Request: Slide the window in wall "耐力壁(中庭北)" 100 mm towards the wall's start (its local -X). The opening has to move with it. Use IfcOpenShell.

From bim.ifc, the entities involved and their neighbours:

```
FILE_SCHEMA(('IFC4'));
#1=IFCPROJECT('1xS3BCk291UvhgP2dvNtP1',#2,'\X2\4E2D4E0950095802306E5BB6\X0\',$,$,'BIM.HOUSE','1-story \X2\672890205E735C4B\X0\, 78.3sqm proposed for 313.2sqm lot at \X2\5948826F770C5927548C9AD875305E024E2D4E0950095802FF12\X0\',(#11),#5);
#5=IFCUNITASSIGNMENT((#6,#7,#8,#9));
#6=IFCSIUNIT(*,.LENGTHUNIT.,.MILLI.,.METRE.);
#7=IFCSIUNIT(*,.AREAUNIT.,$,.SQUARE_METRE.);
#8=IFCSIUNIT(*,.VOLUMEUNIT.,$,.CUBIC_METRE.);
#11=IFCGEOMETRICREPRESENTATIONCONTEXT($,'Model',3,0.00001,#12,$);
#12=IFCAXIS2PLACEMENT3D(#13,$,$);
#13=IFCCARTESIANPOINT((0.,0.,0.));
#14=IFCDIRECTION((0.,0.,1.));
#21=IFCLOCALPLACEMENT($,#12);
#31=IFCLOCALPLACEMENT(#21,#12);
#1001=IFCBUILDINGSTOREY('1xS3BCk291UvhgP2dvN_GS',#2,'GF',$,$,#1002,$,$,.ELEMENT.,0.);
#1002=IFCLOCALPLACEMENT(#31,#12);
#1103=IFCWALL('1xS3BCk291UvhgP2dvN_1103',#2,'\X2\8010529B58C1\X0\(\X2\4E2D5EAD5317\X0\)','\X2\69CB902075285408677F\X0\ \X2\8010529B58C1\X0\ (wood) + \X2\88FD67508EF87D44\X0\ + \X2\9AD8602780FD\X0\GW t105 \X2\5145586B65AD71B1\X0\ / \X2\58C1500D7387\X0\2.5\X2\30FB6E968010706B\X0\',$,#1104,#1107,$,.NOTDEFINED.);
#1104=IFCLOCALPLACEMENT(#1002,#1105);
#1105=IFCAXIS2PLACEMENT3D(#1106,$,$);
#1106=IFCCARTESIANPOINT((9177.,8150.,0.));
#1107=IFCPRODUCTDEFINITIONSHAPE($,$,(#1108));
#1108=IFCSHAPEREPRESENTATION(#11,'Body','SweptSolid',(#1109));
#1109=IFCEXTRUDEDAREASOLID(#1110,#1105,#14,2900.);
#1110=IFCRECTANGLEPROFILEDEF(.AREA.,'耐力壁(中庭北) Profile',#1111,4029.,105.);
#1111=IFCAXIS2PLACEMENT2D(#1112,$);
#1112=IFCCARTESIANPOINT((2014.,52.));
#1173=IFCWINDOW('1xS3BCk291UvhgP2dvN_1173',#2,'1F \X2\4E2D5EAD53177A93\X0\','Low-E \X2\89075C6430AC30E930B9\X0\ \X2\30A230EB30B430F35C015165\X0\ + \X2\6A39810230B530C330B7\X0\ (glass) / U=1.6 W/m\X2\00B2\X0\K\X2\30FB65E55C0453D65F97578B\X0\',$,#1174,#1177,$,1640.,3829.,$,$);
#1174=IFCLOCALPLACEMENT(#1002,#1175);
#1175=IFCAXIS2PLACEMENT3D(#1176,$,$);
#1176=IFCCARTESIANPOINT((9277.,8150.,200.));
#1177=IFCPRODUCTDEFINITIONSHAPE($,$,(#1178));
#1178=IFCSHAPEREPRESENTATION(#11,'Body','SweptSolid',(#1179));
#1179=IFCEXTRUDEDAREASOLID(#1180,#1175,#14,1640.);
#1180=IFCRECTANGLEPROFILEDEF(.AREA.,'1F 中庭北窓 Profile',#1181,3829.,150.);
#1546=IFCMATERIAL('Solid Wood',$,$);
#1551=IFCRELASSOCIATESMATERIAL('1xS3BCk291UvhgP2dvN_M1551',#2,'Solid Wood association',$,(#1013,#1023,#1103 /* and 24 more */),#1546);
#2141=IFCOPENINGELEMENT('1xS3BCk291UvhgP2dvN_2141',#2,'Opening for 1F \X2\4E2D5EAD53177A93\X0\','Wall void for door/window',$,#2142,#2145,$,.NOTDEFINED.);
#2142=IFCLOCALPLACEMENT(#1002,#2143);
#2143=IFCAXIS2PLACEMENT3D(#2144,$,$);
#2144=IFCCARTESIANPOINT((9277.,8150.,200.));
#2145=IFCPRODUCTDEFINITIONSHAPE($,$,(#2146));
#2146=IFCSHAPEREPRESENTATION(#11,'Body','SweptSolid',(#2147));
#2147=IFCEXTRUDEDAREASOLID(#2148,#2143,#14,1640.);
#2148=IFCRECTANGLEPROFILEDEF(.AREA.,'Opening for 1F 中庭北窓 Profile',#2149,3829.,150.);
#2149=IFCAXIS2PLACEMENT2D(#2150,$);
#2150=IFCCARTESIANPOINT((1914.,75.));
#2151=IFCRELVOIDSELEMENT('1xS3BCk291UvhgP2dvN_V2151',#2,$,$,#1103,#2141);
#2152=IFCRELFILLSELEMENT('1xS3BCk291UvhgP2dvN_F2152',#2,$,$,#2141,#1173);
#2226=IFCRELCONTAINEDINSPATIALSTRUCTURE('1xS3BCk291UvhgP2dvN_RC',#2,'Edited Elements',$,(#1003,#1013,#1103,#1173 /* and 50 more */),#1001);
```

```python
import ifcopenshell
import ifcopenshell.api.geometry
import ifcopenshell.util.placement
import ifcopenshell.util.unit

model = ifcopenshell.open("bim.ifc")
unit_scale = ifcopenshell.util.unit.calculate_unit_scale(model)

window = model.by_guid("1xS3BCk291UvhgP2dvN_1173")
opening = window.FillsVoids[0].RelatingOpeningElement
wall = opening.VoidsElements[0].RelatingBuildingElement

wall_matrix = ifcopenshell.util.placement.get_local_placement(wall.ObjectPlacement)
shift = wall_matrix[:3, 0] * -0.1 / unit_scale
before = ifcopenshell.util.placement.get_local_placement(window.ObjectPlacement)[:3, 3].copy()

# The window is not placed relative to its opening, so move both.
for product in (opening, window):
    matrix = ifcopenshell.util.placement.get_local_placement(product.ObjectPlacement)
    matrix[:3, 3] += shift
    ifcopenshell.api.geometry.edit_object_placement(model, product=product, matrix=matrix, is_si=False)

after = ifcopenshell.util.placement.get_local_placement(window.ObjectPlacement)[:3, 3]
print("window moved by", (after - before).round(3) + 0.0)

model.write("bim_updated.ifc")
```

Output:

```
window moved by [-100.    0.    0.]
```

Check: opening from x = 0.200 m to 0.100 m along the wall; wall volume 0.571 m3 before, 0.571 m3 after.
